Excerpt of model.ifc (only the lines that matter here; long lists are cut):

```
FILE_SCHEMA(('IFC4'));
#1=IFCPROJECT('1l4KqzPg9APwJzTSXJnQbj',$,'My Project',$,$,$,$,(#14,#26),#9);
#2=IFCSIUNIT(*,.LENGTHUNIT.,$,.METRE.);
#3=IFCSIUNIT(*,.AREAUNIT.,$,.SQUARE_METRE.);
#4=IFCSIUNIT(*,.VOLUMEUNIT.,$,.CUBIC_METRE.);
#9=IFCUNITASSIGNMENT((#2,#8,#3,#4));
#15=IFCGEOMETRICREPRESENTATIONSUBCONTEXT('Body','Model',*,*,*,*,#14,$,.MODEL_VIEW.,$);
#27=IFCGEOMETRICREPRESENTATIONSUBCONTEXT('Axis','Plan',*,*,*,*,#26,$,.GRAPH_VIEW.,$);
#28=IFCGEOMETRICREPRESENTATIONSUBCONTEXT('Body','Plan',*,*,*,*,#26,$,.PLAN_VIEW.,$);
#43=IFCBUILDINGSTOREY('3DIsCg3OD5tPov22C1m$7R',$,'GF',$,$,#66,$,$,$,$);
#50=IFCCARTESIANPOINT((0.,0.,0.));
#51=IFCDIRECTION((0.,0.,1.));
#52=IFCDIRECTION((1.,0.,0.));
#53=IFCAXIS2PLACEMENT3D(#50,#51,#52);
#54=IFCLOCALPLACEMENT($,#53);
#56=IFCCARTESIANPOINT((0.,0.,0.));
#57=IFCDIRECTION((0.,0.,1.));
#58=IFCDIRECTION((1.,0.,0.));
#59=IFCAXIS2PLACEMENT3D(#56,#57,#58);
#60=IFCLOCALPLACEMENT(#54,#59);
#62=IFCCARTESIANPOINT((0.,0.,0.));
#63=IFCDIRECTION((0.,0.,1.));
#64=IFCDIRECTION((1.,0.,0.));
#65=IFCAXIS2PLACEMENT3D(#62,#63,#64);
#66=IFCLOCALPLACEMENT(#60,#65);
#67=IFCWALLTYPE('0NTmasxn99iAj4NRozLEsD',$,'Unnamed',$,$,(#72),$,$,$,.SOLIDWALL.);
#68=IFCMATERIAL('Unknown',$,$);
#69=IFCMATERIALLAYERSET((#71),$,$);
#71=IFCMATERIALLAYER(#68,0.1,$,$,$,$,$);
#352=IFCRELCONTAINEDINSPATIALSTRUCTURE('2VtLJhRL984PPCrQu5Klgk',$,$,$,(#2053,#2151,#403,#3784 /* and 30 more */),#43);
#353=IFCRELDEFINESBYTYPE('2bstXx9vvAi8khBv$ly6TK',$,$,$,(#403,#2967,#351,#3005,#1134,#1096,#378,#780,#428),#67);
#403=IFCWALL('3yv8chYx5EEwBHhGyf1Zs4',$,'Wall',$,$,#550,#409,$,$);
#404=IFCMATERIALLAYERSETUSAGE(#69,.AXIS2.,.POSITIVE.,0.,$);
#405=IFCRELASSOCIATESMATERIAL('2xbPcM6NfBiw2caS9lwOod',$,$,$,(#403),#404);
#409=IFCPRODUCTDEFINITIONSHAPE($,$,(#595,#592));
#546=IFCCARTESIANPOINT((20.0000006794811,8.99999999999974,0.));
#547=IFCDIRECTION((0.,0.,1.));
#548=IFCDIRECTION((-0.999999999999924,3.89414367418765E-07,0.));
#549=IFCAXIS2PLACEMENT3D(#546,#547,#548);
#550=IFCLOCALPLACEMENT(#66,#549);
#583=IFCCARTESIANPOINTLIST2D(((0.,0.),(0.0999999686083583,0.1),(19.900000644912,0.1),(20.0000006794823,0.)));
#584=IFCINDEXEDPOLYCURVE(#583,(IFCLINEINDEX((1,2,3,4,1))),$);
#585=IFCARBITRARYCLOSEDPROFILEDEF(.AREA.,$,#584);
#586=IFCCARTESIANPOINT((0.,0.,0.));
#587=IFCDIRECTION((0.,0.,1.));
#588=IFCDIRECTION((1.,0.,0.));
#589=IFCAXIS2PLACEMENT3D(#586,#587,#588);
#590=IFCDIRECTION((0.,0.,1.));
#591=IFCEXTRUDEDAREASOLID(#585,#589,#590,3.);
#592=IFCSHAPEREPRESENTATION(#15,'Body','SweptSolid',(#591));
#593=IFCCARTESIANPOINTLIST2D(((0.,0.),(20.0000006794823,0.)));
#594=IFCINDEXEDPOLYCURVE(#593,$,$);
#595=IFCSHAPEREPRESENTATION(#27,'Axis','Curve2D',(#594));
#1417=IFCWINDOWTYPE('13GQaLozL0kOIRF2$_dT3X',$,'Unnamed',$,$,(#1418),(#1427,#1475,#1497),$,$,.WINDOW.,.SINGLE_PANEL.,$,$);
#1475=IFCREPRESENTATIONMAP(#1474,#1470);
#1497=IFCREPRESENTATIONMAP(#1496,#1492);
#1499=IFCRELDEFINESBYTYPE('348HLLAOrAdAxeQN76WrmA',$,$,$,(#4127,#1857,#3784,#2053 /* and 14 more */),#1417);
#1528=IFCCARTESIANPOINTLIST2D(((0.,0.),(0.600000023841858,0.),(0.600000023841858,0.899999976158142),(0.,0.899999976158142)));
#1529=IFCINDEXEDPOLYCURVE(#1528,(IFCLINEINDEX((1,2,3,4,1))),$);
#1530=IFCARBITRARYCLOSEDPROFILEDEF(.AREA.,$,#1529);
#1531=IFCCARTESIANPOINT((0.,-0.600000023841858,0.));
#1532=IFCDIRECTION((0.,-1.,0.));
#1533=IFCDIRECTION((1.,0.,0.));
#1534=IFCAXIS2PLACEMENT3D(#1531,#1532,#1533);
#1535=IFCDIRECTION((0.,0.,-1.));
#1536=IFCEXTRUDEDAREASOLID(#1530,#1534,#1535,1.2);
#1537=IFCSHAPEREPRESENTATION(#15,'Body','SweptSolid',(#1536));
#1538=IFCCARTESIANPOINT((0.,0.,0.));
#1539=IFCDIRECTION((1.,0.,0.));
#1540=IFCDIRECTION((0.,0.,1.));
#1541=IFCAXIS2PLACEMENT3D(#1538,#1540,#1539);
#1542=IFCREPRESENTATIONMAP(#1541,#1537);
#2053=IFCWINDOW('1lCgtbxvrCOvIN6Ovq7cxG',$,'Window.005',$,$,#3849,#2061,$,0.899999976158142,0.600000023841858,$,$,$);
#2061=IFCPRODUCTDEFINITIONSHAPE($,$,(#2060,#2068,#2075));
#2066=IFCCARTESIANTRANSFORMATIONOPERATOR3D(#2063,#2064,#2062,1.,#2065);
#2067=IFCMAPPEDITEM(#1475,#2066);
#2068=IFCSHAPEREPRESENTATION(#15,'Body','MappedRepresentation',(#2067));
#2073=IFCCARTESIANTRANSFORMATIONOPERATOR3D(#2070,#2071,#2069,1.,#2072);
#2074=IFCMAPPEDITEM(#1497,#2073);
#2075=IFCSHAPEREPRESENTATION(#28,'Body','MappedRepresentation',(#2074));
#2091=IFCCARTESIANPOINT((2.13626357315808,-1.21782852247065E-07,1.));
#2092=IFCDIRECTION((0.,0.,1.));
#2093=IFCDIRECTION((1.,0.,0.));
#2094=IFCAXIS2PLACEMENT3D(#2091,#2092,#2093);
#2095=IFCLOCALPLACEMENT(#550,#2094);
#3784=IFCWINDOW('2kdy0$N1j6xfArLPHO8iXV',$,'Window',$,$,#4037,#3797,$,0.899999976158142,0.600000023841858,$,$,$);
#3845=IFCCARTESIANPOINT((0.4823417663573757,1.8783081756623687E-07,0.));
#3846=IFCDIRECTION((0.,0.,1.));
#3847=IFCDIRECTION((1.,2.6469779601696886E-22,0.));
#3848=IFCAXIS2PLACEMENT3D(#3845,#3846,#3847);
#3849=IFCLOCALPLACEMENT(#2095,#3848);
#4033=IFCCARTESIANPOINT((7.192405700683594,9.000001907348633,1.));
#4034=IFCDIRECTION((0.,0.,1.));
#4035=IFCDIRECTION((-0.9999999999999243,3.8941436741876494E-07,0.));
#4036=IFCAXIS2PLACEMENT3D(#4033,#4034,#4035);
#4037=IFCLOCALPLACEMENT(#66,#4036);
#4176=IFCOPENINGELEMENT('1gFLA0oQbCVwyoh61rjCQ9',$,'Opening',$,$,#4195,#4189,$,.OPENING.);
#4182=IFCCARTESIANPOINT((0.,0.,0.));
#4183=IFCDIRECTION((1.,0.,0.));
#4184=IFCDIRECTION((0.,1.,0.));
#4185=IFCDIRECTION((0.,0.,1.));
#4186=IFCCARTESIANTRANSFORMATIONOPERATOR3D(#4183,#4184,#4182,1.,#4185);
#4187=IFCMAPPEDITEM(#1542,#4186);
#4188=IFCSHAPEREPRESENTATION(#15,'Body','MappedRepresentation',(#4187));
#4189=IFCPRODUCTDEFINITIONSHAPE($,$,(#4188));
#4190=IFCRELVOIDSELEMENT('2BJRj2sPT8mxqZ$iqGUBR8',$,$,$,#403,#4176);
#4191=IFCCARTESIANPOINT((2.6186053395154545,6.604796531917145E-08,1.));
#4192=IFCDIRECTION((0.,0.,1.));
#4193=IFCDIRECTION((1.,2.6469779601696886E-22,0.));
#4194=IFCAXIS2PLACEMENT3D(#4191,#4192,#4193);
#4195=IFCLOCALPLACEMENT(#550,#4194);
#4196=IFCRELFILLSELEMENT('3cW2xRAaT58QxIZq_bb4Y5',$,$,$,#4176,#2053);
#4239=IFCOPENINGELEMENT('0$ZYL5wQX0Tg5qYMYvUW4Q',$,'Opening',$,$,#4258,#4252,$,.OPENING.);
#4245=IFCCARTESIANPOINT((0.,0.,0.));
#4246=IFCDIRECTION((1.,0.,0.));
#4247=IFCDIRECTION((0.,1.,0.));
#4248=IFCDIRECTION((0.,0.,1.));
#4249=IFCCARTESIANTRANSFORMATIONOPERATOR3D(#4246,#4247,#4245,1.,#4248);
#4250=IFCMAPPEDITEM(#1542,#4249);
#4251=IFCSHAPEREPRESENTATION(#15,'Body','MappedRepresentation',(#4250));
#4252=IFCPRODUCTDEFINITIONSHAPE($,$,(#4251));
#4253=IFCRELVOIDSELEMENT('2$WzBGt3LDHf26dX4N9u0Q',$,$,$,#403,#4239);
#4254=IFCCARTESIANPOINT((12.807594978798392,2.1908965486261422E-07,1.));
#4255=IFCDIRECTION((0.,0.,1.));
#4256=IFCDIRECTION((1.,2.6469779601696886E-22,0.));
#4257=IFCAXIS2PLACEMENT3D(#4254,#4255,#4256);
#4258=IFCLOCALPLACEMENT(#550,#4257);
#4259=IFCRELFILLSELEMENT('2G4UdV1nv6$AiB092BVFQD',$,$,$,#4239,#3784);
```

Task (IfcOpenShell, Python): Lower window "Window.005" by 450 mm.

```python
import numpy as np
import ifcopenshell
import ifcopenshell.api.geometry
import ifcopenshell.util.placement
import ifcopenshell.util.unit

model = ifcopenshell.open("model.ifc")
unit_scale = ifcopenshell.util.unit.calculate_unit_scale(model)

window = model.by_guid("1lCgtbxvrCOvIN6Ovq7cxG")
opening = window.FillsVoids[0].RelatingOpeningElement
dz = -0.45

shift = np.array([0.0, 0.0, dz])
# The window is not placed relative to its opening, so move both.
for product in (opening, window):
    matrix = ifcopenshell.util.placement.get_local_placement(product.ObjectPlacement)
    matrix[:3, 3] += shift
    ifcopenshell.api.geometry.edit_object_placement(model, product=product, matrix=matrix, is_si=False)

print(f"moved by {dz * unit_scale:+.3f} m")

model.write("model-out.ifc")
```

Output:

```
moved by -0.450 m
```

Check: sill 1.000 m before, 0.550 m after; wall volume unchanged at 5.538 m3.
